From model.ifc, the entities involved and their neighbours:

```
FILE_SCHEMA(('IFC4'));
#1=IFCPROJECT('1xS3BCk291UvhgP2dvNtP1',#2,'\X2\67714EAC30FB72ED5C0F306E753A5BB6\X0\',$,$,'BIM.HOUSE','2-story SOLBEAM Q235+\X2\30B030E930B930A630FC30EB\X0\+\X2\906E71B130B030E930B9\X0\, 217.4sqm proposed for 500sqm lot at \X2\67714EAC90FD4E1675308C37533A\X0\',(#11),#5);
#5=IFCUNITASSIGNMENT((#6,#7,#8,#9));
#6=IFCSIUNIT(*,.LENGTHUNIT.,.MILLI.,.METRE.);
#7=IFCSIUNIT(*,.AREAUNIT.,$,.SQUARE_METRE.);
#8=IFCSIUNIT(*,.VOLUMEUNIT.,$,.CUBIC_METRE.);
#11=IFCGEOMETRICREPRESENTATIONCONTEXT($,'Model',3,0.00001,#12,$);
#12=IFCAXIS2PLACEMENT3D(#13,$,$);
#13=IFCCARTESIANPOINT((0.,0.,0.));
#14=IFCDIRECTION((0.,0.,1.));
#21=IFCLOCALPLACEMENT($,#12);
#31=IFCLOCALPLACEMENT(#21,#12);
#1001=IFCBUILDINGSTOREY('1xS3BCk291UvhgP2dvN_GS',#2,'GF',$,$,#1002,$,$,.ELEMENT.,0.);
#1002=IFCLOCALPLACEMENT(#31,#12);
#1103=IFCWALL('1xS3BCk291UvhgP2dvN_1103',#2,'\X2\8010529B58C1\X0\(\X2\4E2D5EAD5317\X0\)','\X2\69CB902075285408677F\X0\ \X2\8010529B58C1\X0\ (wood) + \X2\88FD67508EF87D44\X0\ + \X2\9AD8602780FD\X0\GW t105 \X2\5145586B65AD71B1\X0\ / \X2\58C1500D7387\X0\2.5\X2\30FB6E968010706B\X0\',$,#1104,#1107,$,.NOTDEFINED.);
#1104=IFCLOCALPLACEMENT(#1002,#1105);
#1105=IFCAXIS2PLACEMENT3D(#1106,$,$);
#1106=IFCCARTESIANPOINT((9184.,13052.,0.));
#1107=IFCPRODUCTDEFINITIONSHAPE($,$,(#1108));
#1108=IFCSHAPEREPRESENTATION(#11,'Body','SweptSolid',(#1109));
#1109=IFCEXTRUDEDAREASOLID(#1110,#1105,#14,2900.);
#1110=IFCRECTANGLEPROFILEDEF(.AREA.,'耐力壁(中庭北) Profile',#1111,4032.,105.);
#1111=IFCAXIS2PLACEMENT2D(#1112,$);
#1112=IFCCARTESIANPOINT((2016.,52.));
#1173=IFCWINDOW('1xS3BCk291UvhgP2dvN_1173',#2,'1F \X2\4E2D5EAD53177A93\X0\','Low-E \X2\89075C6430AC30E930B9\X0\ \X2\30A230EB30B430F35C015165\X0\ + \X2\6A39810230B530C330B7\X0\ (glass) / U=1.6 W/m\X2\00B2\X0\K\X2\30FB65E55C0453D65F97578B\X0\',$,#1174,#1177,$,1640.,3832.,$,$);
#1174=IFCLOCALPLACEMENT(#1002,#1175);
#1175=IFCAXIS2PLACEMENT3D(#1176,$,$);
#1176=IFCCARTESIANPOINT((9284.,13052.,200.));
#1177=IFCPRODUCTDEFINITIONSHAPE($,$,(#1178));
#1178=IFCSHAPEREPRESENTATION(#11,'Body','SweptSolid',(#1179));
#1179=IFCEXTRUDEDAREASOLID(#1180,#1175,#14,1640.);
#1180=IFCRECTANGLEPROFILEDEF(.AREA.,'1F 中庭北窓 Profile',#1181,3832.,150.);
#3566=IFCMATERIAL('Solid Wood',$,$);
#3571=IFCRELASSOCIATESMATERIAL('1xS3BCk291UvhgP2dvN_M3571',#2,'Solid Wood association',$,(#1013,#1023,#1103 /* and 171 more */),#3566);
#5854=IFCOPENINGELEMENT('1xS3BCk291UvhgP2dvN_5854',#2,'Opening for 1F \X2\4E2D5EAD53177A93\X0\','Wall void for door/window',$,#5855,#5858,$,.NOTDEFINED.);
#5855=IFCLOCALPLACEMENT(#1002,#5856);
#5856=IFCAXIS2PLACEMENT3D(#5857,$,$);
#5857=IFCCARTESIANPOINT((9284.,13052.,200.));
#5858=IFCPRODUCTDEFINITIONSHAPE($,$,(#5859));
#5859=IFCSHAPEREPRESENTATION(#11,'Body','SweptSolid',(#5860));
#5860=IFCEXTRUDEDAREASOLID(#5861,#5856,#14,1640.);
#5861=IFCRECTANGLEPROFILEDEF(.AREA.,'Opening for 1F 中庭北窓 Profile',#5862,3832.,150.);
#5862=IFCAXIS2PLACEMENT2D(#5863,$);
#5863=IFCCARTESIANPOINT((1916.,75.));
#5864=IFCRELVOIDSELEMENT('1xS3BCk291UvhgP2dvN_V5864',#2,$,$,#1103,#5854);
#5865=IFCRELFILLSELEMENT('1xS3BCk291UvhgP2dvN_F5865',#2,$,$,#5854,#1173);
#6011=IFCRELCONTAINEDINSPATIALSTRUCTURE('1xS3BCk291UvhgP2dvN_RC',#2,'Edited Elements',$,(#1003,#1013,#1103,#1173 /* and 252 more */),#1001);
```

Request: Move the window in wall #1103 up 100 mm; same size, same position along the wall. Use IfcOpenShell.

```python
import numpy as np
import ifcopenshell
import ifcopenshell.api.geometry
import ifcopenshell.util.placement
import ifcopenshell.util.unit

model = ifcopenshell.open("model.ifc")
unit_scale = ifcopenshell.util.unit.calculate_unit_scale(model)

window = model.by_guid("1xS3BCk291UvhgP2dvN_1173")
opening = window.FillsVoids[0].RelatingOpeningElement
dz = 0.1 / unit_scale

shift = np.array([0.0, 0.0, dz])
# The window is not placed relative to its opening, so move both.
for product in (opening, window):
    matrix = ifcopenshell.util.placement.get_local_placement(product.ObjectPlacement)
    matrix[:3, 3] += shift
    ifcopenshell.api.geometry.edit_object_placement(model, product=product, matrix=matrix, is_si=False)

print(f"moved by {dz * unit_scale:+.3f} m")

model.write("model_v2.ifc")
```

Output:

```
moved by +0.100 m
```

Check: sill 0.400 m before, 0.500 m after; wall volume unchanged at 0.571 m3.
